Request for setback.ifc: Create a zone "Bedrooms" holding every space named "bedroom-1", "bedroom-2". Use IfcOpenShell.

First a look at what the model holds.

```python
import ifcopenshell

model = ifcopenshell.open("setback.ifc")
print(model.schema)
seen = {}
for space in model.by_type("IfcSpace"):
    seen[space.Name] = seen.get(space.Name, 0) + 1
for name, count in sorted(seen.items(), key=str):
    print(count, "x", name)
print("zones:", [z.Name for z in model.by_type("IfcZone")][:20])
```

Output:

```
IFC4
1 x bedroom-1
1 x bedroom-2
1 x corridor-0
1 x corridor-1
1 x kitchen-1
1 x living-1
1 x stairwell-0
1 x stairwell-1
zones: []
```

```python
import ifcopenshell
import ifcopenshell.api.group
import ifcopenshell.api.root

model = ifcopenshell.open("setback.ifc")

names = {"bedroom-1", "bedroom-2"}
spaces = [s for s in model.by_type("IfcSpace") if s.Name in names]

zone = ifcopenshell.api.root.create_entity(model, ifc_class="IfcZone", name="Bedrooms")
ifcopenshell.api.group.assign_group(model, products=spaces, group=zone)
print(len(spaces), "spaces in", zone.Name)

model.write("setback_updated.ifc")
```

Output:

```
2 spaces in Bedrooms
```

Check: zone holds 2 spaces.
